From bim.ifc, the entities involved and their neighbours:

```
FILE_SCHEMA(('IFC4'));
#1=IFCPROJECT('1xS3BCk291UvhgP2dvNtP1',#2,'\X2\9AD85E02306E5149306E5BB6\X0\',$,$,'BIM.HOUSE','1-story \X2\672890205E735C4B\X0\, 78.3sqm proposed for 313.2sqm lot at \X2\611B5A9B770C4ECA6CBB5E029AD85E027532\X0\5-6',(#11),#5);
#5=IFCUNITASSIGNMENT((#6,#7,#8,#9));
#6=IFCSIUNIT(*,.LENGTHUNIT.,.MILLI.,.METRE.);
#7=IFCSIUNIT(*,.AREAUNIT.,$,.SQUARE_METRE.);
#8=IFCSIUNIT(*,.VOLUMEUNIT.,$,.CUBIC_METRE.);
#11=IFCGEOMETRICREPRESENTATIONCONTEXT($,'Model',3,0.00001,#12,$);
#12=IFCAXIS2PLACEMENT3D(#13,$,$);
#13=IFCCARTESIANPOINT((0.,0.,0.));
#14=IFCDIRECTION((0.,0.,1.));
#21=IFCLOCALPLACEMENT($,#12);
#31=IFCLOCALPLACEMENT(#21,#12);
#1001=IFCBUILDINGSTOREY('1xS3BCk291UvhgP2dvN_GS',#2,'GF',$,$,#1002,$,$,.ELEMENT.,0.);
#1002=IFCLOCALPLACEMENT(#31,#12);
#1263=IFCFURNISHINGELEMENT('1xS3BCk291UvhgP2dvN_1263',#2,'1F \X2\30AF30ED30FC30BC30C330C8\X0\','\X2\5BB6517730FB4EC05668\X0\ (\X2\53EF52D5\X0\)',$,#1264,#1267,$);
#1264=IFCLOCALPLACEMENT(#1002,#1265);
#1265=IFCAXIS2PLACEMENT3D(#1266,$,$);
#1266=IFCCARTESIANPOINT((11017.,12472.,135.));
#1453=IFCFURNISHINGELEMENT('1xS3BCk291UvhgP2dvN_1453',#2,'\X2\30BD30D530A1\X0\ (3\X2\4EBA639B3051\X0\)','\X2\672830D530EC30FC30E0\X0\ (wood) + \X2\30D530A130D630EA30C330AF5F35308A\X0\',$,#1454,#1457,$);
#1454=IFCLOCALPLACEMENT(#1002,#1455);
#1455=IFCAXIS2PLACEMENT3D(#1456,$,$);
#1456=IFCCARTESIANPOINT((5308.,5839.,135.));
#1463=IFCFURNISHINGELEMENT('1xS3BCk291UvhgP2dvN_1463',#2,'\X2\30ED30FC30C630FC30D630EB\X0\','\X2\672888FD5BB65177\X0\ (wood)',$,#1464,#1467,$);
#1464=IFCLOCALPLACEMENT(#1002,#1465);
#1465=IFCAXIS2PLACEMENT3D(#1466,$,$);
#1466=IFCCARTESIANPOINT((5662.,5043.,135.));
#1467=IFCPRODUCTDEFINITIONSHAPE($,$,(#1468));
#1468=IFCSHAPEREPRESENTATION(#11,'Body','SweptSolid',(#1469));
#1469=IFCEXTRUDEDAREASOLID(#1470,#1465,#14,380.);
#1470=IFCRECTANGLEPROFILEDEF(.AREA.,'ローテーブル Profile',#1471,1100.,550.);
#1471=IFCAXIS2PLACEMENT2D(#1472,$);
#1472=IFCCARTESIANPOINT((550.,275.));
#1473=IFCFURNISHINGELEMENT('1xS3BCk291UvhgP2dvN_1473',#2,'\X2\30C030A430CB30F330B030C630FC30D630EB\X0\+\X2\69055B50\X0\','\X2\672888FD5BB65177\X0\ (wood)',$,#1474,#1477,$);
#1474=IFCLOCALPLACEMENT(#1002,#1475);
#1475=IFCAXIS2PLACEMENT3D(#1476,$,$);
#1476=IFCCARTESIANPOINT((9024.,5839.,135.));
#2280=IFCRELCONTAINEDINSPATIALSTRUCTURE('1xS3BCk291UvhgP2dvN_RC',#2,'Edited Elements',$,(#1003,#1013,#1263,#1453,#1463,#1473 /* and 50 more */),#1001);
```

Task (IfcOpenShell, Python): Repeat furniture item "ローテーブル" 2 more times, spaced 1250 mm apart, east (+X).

```python
import numpy as np
import ifcopenshell
import ifcopenshell.api.geometry
import ifcopenshell.api.root
import ifcopenshell.util.element
import ifcopenshell.util.placement
import ifcopenshell.util.unit

model = ifcopenshell.open("bim.ifc")
unit_scale = ifcopenshell.util.unit.calculate_unit_scale(model)


def reuse_history(source, copy):
    """copy_class also copies each property set's owner history, people and application; keep the originals."""
    for rel in copy.IsDefinedBy:
        if rel.is_a("IfcRelDefinesByProperties") and (history := rel.RelatingPropertyDefinition.OwnerHistory):
            rel.RelatingPropertyDefinition.OwnerHistory = source.OwnerHistory
            ifcopenshell.util.element.remove_deep2(model, history)


source = model.by_guid("1xS3BCk291UvhgP2dvN_1463")
base = ifcopenshell.util.placement.get_local_placement(source.ObjectPlacement)
step = np.array([1.0, 0.0, 0.0]) * 1.25 / unit_scale

for i in range(1, 3):
    copy = ifcopenshell.api.root.copy_class(model, product=source)
    copy.Representation = ifcopenshell.util.element.copy_deep(
        model, source.Representation, exclude=["IfcGeometricRepresentationContext", "IfcRepresentationMap"]
    )
    reuse_history(source, copy)
    matrix = base.copy()
    matrix[:3, 3] += i * step
    print("added at", matrix[:3, 3].round(3) + 0.0)
    ifcopenshell.api.geometry.edit_object_placement(model, product=copy, matrix=matrix, is_si=False)

model.write("bim_edited.ifc")
```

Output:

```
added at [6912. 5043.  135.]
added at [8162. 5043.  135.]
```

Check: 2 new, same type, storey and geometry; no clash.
